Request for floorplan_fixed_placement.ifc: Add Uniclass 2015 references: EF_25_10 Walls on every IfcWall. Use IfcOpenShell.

First a look at what the model holds.

```python
import ifcopenshell

model = ifcopenshell.open("floorplan_fixed_placement.ifc")
print(model.schema)
print("classifications:", [c.Name for c in model.by_type("IfcClassification")])
for ifc_class in ("IfcDoor", "IfcRoof", "IfcStair", "IfcWall", "IfcWindow"):
    print(ifc_class, len(model.by_type(ifc_class)))
```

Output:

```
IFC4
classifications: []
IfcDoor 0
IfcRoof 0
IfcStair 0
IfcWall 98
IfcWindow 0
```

```python
import ifcopenshell
import ifcopenshell.api.classification

model = ifcopenshell.open("floorplan_fixed_placement.ifc")

system = ifcopenshell.api.classification.add_classification(model, classification="Uniclass 2015")

codes = {
    "IfcWall": ("EF_25_10", "Walls"),
}
for ifc_class, (code, name) in codes.items():
    products = model.by_type(ifc_class)
    ifcopenshell.api.classification.add_reference(
        model, products=products, classification=system, identification=code, name=name
    )
    print(code, len(products))

model.write("floorplan_fixed_placement_v2.ifc")
```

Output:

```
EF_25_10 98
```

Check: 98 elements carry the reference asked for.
